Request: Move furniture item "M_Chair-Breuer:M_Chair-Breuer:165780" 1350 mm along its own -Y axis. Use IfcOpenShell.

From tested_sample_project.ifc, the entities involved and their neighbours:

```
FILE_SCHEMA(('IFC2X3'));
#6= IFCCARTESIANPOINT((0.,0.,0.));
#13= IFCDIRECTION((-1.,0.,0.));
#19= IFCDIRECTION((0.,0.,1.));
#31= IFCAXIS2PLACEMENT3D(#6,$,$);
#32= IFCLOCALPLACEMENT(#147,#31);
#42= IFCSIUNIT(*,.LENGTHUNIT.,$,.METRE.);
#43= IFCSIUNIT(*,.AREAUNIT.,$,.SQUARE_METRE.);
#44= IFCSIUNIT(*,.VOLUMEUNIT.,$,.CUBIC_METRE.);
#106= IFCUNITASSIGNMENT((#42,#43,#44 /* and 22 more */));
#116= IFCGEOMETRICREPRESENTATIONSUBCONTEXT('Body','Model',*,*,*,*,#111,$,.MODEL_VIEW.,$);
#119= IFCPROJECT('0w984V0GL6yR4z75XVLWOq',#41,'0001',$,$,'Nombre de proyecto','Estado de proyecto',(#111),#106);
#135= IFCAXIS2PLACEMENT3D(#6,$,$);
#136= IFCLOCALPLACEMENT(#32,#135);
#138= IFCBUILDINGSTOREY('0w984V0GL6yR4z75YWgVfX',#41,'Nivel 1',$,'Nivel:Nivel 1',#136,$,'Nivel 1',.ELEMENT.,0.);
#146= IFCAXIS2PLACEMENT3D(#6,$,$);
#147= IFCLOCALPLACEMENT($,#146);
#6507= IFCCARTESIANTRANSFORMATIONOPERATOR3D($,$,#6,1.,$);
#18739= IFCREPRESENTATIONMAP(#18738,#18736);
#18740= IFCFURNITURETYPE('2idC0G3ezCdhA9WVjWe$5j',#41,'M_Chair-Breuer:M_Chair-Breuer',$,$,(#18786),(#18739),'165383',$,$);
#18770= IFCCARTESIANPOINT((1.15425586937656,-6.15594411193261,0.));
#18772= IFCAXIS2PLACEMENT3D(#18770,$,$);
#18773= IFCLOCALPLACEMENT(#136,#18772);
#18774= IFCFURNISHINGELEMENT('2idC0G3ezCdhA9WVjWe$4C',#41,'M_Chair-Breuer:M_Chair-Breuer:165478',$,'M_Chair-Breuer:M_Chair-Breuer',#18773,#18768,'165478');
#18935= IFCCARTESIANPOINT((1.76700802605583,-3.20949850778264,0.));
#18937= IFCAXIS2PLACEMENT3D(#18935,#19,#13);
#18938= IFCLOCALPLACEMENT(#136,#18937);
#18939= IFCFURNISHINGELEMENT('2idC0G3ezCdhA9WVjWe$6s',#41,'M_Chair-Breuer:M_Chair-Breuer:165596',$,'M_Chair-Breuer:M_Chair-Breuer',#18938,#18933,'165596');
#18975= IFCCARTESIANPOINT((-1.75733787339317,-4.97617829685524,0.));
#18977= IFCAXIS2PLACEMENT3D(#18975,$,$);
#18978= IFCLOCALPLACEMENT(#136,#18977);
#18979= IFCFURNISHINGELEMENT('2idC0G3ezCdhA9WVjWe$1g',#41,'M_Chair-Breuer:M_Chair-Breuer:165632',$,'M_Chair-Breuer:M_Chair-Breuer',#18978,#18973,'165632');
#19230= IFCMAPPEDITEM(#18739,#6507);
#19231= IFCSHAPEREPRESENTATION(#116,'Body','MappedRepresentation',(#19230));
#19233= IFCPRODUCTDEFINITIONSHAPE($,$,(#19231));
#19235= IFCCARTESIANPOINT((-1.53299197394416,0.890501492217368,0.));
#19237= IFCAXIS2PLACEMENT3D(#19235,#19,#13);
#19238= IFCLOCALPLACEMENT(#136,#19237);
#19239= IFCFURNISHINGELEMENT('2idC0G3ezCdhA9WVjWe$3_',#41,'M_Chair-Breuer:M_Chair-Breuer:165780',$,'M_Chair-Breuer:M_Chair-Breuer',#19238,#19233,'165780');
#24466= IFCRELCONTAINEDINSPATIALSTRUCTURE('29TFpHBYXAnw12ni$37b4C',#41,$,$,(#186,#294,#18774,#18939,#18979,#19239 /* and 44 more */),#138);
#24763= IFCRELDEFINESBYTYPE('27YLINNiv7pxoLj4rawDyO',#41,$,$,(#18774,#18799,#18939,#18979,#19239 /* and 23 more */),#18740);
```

```python
import ifcopenshell
import ifcopenshell.api.geometry
import ifcopenshell.util.placement
import ifcopenshell.util.unit

model = ifcopenshell.open("tested_sample_project.ifc")
unit_scale = ifcopenshell.util.unit.calculate_unit_scale(model)

item = model.by_guid("2idC0G3ezCdhA9WVjWe$3_")
matrix = ifcopenshell.util.placement.get_local_placement(item.ObjectPlacement)
matrix[:3, 3] -= matrix[:3, 1] * 1.35 / unit_scale
ifcopenshell.api.geometry.edit_object_placement(model, product=item, matrix=matrix, is_si=False)

print(ifcopenshell.util.placement.get_local_placement(item.ObjectPlacement).round(3) + 0.0)

model.write("tested_sample_project_v2.ifc")
```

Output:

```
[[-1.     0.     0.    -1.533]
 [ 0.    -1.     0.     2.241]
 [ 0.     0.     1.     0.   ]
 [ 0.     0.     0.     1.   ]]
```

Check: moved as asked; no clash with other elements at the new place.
